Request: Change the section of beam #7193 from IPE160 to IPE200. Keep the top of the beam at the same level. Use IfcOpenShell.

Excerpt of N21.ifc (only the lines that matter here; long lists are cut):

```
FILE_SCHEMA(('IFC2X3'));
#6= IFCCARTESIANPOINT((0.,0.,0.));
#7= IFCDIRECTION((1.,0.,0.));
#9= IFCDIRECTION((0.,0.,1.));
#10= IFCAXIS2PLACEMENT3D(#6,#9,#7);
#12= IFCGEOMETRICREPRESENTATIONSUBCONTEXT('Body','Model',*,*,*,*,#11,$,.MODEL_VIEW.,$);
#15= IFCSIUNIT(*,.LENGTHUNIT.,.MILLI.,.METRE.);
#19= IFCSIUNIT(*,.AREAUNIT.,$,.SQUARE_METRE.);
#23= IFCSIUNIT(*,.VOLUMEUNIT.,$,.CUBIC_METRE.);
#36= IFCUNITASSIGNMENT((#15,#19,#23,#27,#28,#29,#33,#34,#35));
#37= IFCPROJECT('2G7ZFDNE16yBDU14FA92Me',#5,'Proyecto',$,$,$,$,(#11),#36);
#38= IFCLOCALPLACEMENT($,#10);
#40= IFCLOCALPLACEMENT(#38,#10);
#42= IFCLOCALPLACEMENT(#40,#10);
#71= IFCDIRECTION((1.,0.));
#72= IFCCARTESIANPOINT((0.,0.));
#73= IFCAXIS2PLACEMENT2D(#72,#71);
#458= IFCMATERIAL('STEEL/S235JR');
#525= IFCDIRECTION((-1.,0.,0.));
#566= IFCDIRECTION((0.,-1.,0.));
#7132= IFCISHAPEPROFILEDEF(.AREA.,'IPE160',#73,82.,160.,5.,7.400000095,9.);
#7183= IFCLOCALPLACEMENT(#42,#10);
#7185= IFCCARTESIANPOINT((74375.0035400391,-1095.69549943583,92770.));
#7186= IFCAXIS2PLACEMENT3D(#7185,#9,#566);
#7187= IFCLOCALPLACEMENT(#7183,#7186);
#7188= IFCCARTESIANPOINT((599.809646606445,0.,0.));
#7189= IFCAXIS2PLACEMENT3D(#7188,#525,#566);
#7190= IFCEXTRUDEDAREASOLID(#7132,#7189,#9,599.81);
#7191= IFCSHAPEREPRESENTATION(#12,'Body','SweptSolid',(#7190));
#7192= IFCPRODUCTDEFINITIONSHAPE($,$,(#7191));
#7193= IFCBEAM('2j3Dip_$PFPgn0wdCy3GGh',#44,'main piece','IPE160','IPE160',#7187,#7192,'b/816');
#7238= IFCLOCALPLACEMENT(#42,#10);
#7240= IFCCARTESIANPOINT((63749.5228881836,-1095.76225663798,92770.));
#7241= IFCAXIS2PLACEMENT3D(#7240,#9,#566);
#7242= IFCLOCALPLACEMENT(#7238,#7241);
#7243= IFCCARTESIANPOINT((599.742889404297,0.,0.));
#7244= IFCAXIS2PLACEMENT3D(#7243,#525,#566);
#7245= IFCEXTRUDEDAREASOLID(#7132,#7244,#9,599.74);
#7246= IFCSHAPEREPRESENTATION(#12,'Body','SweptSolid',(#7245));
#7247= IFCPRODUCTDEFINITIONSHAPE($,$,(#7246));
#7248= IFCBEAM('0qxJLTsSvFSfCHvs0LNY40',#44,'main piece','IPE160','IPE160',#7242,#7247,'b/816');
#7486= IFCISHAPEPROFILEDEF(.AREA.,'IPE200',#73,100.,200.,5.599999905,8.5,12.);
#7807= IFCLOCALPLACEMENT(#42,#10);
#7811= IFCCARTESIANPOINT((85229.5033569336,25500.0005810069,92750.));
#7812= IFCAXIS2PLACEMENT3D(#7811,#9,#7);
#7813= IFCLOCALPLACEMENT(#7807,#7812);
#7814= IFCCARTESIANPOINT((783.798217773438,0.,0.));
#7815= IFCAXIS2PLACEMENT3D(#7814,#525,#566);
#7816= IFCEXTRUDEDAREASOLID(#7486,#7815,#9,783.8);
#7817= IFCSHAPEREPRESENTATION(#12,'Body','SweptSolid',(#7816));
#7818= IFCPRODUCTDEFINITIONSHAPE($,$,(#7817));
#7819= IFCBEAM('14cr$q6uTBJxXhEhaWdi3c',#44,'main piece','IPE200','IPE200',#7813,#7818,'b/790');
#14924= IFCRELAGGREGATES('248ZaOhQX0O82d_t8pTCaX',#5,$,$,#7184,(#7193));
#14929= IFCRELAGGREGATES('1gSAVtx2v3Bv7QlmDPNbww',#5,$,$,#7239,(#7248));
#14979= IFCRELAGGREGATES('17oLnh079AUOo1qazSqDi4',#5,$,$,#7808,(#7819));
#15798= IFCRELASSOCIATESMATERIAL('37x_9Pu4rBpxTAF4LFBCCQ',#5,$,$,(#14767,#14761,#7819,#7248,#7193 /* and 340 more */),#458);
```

```python
import ifcopenshell
import ifcopenshell.util.element
import ifcopenshell.util.representation

model = ifcopenshell.open("N21.ifc")

member = model.by_guid("2j3Dip_$PFPgn0wdCy3GGh")
source = next(p for p in model.by_type("IfcIShapeProfileDef") if p.ProfileName == "IPE200")

body = ifcopenshell.util.representation.get_representation(member, "Model", "Body")
solid = body.Items[0]
old_profile = solid.SweptArea

# Copy the section's sizes but keep this member's own profile position.
profile = ifcopenshell.util.element.copy(model, source)
# Profiles are centred, so shift by half the change in depth to hold the top.
shift = (old_profile.OverallDepth - profile.OverallDepth) / 2
x, y = old_profile.Position.Location.Coordinates
up = (0.0, 1.0)  # upwards, in the solid's own plane
location = model.createIfcCartesianPoint((x + up[0] * shift, y + up[1] * shift))
profile.Position = model.createIfcAxis2Placement2D(location, old_profile.Position.RefDirection)
solid.SweptArea = profile
if not model.get_total_inverses(old_profile):
    ifcopenshell.util.element.remove_deep2(model, old_profile)
member.Description = member.Description.replace("IPE160", "IPE200")
member.ObjectType = member.ObjectType.replace("IPE160", "IPE200")

print(solid.SweptArea)

model.write("N21_rev.ifc")
```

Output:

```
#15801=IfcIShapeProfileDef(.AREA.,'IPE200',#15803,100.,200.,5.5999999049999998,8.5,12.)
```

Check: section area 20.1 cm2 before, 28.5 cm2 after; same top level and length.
